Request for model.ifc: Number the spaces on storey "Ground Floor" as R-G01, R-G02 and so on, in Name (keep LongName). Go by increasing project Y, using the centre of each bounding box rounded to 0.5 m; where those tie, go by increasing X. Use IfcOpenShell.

First a look at what the model holds.

```python
import ifcopenshell
import ifcopenshell.util.element
import ifcopenshell.util.placement

model = ifcopenshell.open("model.ifc")
print(model.schema)
storey = next(s for s in model.by_type("IfcBuildingStorey") if s.Name == "Ground Floor")
spaces = [e for e in ifcopenshell.util.element.get_decomposition(storey) if e.is_a("IfcSpace")]
for e in sorted(spaces, key=lambda e: e.id()):
    origin = ifcopenshell.util.placement.get_local_placement(e.ObjectPlacement)[:3, 3]
    print(e.id(), e.Name, e.LongName, origin.round(2) + 0.0, sep=" | ")
```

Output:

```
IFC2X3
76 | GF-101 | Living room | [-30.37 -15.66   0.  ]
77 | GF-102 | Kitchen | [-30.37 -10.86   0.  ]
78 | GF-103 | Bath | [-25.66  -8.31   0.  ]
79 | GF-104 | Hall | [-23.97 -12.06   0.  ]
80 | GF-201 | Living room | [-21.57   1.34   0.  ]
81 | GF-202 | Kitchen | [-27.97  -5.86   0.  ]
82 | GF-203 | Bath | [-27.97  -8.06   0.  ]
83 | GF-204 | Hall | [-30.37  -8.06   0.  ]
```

```python
import ifcopenshell
import ifcopenshell.geom
import ifcopenshell.util.element
import ifcopenshell.util.shape

model = ifcopenshell.open("model.ifc")
settings = ifcopenshell.geom.settings()
settings.set("use-world-coords", True)


def centre(element):
    shape = ifcopenshell.geom.create_shape(settings, element)
    return ifcopenshell.util.shape.get_bbox_centroid(shape.geometry)


storey = next(s for s in model.by_type("IfcBuildingStorey") if s.Name == "Ground Floor")
spaces = [e for e in ifcopenshell.util.element.get_decomposition(storey) if e.is_a("IfcSpace")]

# Insertion points can sit at a corner or the storey origin, so sort by the geometry (in metres).
centres = {e: centre(e) for e in spaces}
spaces.sort(key=lambda e: (round(centres[e][1] / 0.5), centres[e][0]))

for i, e in enumerate(spaces, start=1):
    number = f"R-G{i:02d}"
    e.Name = number
    print(e.id(), number)

model.write("model_updated.ifc")
```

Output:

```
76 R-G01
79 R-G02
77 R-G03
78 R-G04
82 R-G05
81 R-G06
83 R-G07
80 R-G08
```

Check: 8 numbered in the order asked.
